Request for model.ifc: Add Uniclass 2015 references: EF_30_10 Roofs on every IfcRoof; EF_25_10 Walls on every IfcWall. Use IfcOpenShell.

First a look at what the model holds.

```python
import ifcopenshell

model = ifcopenshell.open("model.ifc")
print(model.schema)
print("classifications:", [c.Name for c in model.by_type("IfcClassification")])
for ifc_class in ("IfcDoor", "IfcRoof", "IfcStair", "IfcWall", "IfcWindow"):
    print(ifc_class, len(model.by_type(ifc_class)))
```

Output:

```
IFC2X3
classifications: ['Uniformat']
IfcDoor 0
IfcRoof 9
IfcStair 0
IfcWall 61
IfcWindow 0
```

```python
import ifcopenshell
import ifcopenshell.api.classification

model = ifcopenshell.open("model.ifc")

# IFC2X3 requires Source and Edition and has no link from the project to the system.
system = model.create_entity("IfcClassification", Source="NBS", Edition="2015", Name="Uniclass 2015")

codes = {
    "IfcRoof": ("EF_30_10", "Roofs"),
    "IfcWall": ("EF_25_10", "Walls"),
}
for ifc_class, (code, name) in codes.items():
    products = model.by_type(ifc_class)
    ifcopenshell.api.classification.add_reference(
        model, products=products, classification=system, identification=code, name=name
    )
    print(code, len(products))

model.write("model_v2.ifc")
```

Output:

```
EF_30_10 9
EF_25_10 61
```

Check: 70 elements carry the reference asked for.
